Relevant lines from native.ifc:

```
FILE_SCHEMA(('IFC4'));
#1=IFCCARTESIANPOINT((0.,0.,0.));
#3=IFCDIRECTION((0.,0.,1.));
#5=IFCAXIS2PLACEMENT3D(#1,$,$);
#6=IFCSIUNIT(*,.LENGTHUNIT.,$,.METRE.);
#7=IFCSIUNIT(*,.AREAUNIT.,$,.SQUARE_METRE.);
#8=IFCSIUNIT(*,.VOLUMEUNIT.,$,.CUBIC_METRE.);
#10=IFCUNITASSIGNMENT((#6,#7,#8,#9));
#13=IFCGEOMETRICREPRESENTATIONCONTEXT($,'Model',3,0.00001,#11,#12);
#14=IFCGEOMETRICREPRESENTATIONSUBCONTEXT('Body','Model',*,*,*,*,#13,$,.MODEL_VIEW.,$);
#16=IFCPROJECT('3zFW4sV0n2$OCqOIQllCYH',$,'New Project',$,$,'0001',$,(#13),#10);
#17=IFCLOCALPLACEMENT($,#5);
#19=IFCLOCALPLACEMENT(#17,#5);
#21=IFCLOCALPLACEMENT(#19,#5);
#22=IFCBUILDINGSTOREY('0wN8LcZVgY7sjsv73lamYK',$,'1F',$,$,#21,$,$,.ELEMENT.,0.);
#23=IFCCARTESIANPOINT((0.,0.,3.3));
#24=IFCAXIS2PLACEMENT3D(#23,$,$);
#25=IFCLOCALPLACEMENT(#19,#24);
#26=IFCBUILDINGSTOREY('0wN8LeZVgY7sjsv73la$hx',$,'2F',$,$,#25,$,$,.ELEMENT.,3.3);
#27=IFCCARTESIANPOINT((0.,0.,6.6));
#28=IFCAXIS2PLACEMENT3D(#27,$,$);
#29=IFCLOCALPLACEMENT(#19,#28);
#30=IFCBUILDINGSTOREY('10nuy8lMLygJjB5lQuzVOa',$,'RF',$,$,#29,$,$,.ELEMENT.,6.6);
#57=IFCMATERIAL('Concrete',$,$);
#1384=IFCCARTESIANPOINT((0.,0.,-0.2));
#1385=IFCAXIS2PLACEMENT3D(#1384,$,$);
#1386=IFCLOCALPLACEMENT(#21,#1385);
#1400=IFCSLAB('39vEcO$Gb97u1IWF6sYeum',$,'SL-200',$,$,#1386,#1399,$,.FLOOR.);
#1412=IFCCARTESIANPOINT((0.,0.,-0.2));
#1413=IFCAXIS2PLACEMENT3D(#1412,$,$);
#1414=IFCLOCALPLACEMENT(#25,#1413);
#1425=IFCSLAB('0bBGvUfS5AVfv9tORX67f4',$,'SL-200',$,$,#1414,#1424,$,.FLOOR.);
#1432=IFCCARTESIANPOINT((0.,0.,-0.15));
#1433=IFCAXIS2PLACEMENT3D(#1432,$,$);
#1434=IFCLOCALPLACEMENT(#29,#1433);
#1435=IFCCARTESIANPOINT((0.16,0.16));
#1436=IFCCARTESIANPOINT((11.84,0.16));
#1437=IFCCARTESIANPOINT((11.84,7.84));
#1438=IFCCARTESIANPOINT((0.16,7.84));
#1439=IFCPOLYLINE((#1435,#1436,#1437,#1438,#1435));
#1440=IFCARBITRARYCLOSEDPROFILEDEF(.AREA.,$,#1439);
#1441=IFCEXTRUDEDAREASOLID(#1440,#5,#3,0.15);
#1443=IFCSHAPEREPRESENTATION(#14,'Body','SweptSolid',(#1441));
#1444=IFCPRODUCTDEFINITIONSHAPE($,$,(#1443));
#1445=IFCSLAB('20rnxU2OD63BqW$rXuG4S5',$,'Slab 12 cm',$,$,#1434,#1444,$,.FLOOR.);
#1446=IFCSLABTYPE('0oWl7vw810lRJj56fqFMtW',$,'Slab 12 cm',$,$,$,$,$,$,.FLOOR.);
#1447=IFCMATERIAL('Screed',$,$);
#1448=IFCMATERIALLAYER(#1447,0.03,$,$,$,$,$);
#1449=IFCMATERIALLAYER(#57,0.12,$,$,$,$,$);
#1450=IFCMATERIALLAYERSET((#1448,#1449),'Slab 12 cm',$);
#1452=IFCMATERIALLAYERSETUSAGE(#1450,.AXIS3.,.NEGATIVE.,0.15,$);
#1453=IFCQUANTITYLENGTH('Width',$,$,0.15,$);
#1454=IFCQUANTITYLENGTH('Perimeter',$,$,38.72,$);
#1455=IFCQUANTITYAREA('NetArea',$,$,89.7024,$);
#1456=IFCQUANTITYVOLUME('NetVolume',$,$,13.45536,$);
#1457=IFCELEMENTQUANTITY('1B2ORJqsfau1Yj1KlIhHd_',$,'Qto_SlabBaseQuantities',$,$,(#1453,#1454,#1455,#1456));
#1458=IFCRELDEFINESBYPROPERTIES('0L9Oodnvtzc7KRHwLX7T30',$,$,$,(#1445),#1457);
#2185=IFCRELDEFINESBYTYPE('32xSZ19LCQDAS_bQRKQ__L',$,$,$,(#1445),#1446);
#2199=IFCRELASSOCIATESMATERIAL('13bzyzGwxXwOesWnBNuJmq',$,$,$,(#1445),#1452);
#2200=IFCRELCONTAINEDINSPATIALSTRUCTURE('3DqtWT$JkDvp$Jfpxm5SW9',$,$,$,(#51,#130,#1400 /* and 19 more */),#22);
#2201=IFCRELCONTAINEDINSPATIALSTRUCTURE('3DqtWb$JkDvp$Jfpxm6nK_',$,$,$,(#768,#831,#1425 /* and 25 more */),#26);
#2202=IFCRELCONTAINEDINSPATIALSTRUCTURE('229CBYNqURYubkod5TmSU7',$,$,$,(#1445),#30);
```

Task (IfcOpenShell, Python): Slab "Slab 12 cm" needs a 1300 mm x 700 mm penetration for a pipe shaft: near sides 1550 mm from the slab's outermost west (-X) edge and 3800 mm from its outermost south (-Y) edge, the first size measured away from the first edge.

```python
import numpy as np
import ifcopenshell
import ifcopenshell.api.feature
import ifcopenshell.api.geometry
import ifcopenshell.api.pset
import ifcopenshell.api.root
import ifcopenshell.geom
import ifcopenshell.util.element
import ifcopenshell.util.placement
import ifcopenshell.util.representation
import ifcopenshell.util.shape
import ifcopenshell.util.unit

model = ifcopenshell.open("native.ifc")
unit_scale = ifcopenshell.util.unit.calculate_unit_scale(model)
area_scale = ifcopenshell.util.unit.calculate_unit_scale(model, "AREAUNIT")
volume_scale = ifcopenshell.util.unit.calculate_unit_scale(model, "VOLUMEUNIT")
settings = ifcopenshell.geom.settings()


def volume(element):
    """Net volume in cubic metres, openings subtracted."""
    shape = ifcopenshell.geom.create_shape(settings, element)
    return ifcopenshell.util.shape.get_volume(shape.geometry)


slab = model.by_guid("20rnxU2OD63BqW$rXuG4S5")
before = volume(slab)

# Extent in the slab's own axes, in metres. The edges named are its -X and -Y sides.
slab_shape = ifcopenshell.geom.create_shape(settings, slab)
vertices = ifcopenshell.util.shape.get_vertices(slab_shape.geometry)
x_min, y_min, bottom = vertices.min(axis=0)
top = vertices[:, 2].max()

opening = ifcopenshell.api.root.create_entity(model, ifc_class="IfcOpeningElement", name="Pipe shaft opening", predefined_type="OPENING")
context = ifcopenshell.util.representation.get_context(model, "Model", "Body", "MODEL_VIEW")
width, depth = 1.3, 0.7
outline = [(0.0, 0.0), (width, 0.0), (width, depth), (0.0, depth), (0.0, 0.0)]
# Overshoot both faces by 50 mm so the cut is clean.
shape = ifcopenshell.api.geometry.add_slab_representation(
    model, context=context, depth=top - bottom + 0.1, polyline=outline
)
ifcopenshell.api.geometry.assign_representation(model, product=opening, representation=shape)

matrix = ifcopenshell.util.placement.get_local_placement(slab.ObjectPlacement)
matrix[:, 3] = matrix @ np.append(np.array([x_min + 1.55, y_min + 3.8, bottom - 0.05]) / unit_scale, 1.0)
ifcopenshell.api.geometry.edit_object_placement(model, product=opening, matrix=matrix, is_si=False)
ifcopenshell.api.feature.add_feature(model, feature=opening, element=slab)

after = volume(slab)

# Update the slab's stored quantities.
qto = model.by_id(ifcopenshell.util.element.get_pset(slab, "Qto_SlabBaseQuantities", should_inherit=False)["id"])
ifcopenshell.api.pset.edit_qto(model, qto=qto, properties={
    "NetArea": after / (top - bottom) / area_scale,
    "NetVolume": after / volume_scale,
})

print(f"slab volume {before:.3f} -> {after:.3f} m3")

model.write("native_v2.ifc")
```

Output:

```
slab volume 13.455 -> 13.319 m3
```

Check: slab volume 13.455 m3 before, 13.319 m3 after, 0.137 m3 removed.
